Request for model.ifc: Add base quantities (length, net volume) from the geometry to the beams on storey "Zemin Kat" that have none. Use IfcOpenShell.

First a look at what the model holds.

```python
import ifcopenshell
import ifcopenshell.util.element
import ifcopenshell.util.unit

model = ifcopenshell.open("model.ifc")
print(model.schema)
for unit_type in ("LENGTHUNIT", "AREAUNIT", "VOLUMEUNIT"):
    print(unit_type, ifcopenshell.util.unit.calculate_unit_scale(model, unit_type))
storey = next(s for s in model.by_type("IfcBuildingStorey") if s.Name == "Zemin Kat")
beams = [e for e in ifcopenshell.util.element.get_decomposition(storey) if e.is_a("IfcBeam")]
for e in sorted(beams, key=lambda e: e.id()):
    print(e.id(), e.is_a(), e.Name, list(ifcopenshell.util.element.get_psets(e, qtos_only=True)), sep=" | ")
```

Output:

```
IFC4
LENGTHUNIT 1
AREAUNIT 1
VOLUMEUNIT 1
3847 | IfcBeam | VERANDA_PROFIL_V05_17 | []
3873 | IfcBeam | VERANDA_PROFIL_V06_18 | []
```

```python
import ifcopenshell
import ifcopenshell.api.pset
import ifcopenshell.geom
import ifcopenshell.util.element
import ifcopenshell.util.shape
import ifcopenshell.util.unit

model = ifcopenshell.open("model.ifc")
unit_scale = ifcopenshell.util.unit.calculate_unit_scale(model)
volume_scale = ifcopenshell.util.unit.calculate_unit_scale(model, "VOLUMEUNIT")
settings = ifcopenshell.geom.settings()

storey = next(s for s in model.by_type("IfcBuildingStorey") if s.Name == "Zemin Kat")
beams = [e for e in ifcopenshell.util.element.get_decomposition(storey) if e.is_a("IfcBeam")]

for e in sorted(beams, key=lambda e: e.id()):
    if ifcopenshell.util.element.get_psets(e, qtos_only=True, should_inherit=False):
        continue
    # Geometry comes back in metres, in the element's own axes.
    shape = ifcopenshell.geom.create_shape(settings, e)
    values = {
        "Length": ifcopenshell.util.shape.get_max_xyz(shape.geometry) / unit_scale,
        "NetVolume": ifcopenshell.util.shape.get_volume(shape.geometry) / volume_scale,
    }
    qto = ifcopenshell.api.pset.add_qto(model, product=e, name="Qto_BeamBaseQuantities")
    ifcopenshell.api.pset.edit_qto(model, qto=qto, properties=values)
    print(e.id(), {k: round(v, 3) for k, v in values.items()})

model.write("model_rev.ifc")
```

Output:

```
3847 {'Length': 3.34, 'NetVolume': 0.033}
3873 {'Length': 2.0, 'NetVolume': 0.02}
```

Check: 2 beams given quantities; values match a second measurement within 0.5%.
